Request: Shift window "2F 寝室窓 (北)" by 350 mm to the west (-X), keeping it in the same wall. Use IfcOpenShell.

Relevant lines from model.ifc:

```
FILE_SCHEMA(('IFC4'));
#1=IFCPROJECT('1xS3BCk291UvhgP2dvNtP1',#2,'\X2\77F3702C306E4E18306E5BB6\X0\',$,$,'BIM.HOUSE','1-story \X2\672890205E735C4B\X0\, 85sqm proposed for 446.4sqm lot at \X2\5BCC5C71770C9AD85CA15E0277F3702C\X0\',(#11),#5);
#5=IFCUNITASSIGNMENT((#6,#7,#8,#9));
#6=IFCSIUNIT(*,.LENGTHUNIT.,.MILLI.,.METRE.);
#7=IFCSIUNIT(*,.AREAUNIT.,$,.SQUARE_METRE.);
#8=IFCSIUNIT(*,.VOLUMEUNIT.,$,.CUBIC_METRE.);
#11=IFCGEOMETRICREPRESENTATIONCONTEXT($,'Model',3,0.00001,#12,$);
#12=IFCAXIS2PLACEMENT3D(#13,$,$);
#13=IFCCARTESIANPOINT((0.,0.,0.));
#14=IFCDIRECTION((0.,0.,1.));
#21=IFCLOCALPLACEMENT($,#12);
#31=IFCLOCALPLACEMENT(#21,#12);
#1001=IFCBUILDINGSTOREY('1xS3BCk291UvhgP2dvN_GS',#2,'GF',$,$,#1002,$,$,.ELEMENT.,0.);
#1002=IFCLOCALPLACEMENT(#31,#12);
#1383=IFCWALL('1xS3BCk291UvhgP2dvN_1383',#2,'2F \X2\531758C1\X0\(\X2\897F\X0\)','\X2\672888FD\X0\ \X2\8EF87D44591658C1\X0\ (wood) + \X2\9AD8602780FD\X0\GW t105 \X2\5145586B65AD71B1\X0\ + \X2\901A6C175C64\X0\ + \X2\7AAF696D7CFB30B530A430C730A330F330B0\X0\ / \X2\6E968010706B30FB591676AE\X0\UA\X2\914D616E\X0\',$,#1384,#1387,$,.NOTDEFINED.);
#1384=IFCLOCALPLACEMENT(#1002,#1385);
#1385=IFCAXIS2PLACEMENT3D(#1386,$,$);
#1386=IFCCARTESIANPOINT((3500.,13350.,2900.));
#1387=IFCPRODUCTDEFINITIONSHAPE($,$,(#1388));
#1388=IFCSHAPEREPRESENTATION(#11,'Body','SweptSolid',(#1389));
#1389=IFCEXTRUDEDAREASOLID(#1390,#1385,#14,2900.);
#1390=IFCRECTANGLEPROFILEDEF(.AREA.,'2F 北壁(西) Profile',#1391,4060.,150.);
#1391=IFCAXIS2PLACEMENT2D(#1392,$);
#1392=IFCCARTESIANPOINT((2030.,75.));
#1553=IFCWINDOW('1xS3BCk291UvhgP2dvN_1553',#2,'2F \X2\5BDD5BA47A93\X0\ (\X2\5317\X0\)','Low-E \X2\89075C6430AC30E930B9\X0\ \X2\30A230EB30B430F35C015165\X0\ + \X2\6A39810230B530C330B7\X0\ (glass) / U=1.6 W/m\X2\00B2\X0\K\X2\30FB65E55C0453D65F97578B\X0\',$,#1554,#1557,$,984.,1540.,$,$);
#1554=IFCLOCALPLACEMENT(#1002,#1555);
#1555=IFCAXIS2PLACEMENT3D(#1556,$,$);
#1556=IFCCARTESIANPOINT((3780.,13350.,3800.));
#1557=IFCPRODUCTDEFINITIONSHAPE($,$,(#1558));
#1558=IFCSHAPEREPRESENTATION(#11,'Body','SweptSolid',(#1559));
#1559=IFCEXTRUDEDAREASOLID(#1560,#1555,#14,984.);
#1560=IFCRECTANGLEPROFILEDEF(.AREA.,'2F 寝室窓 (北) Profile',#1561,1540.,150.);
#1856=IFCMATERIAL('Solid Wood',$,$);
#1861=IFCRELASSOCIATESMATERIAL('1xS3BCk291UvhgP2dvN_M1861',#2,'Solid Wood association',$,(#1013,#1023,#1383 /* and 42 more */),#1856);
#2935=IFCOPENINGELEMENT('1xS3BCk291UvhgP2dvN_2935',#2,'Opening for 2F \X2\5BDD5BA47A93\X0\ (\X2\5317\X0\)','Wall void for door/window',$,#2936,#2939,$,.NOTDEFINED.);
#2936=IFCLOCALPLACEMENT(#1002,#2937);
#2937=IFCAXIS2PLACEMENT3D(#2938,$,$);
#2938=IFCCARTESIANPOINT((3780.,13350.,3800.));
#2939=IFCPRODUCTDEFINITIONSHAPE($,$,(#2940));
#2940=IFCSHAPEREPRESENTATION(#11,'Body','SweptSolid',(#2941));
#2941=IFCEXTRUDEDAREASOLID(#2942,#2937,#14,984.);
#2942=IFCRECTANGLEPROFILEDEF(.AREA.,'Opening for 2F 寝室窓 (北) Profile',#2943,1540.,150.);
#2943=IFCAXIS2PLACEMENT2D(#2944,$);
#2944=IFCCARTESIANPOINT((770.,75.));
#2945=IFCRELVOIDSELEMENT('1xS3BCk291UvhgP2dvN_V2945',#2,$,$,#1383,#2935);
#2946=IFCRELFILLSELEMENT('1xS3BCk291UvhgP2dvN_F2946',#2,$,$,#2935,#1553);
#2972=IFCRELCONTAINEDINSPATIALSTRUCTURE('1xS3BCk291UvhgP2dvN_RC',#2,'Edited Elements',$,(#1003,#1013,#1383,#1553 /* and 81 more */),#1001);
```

```python
import ifcopenshell
import ifcopenshell.api.geometry
import ifcopenshell.util.placement
import ifcopenshell.util.unit

model = ifcopenshell.open("model.ifc")
unit_scale = ifcopenshell.util.unit.calculate_unit_scale(model)

window = model.by_id(1553)
opening = window.FillsVoids[0].RelatingOpeningElement
wall = opening.VoidsElements[0].RelatingBuildingElement

wall_matrix = ifcopenshell.util.placement.get_local_placement(wall.ObjectPlacement)
shift = wall_matrix[:3, 0] * -0.35 / unit_scale
before = ifcopenshell.util.placement.get_local_placement(window.ObjectPlacement)[:3, 3].copy()

# The window is not placed relative to its opening, so move both.
for product in (opening, window):
    matrix = ifcopenshell.util.placement.get_local_placement(product.ObjectPlacement)
    matrix[:3, 3] += shift
    ifcopenshell.api.geometry.edit_object_placement(model, product=product, matrix=matrix, is_si=False)

after = ifcopenshell.util.placement.get_local_placement(window.ObjectPlacement)[:3, 3]
print("window moved by", (after - before).round(3) + 0.0)

model.write("model-out.ifc")
```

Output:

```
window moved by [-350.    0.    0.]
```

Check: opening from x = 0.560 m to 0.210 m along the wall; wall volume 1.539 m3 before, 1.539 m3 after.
